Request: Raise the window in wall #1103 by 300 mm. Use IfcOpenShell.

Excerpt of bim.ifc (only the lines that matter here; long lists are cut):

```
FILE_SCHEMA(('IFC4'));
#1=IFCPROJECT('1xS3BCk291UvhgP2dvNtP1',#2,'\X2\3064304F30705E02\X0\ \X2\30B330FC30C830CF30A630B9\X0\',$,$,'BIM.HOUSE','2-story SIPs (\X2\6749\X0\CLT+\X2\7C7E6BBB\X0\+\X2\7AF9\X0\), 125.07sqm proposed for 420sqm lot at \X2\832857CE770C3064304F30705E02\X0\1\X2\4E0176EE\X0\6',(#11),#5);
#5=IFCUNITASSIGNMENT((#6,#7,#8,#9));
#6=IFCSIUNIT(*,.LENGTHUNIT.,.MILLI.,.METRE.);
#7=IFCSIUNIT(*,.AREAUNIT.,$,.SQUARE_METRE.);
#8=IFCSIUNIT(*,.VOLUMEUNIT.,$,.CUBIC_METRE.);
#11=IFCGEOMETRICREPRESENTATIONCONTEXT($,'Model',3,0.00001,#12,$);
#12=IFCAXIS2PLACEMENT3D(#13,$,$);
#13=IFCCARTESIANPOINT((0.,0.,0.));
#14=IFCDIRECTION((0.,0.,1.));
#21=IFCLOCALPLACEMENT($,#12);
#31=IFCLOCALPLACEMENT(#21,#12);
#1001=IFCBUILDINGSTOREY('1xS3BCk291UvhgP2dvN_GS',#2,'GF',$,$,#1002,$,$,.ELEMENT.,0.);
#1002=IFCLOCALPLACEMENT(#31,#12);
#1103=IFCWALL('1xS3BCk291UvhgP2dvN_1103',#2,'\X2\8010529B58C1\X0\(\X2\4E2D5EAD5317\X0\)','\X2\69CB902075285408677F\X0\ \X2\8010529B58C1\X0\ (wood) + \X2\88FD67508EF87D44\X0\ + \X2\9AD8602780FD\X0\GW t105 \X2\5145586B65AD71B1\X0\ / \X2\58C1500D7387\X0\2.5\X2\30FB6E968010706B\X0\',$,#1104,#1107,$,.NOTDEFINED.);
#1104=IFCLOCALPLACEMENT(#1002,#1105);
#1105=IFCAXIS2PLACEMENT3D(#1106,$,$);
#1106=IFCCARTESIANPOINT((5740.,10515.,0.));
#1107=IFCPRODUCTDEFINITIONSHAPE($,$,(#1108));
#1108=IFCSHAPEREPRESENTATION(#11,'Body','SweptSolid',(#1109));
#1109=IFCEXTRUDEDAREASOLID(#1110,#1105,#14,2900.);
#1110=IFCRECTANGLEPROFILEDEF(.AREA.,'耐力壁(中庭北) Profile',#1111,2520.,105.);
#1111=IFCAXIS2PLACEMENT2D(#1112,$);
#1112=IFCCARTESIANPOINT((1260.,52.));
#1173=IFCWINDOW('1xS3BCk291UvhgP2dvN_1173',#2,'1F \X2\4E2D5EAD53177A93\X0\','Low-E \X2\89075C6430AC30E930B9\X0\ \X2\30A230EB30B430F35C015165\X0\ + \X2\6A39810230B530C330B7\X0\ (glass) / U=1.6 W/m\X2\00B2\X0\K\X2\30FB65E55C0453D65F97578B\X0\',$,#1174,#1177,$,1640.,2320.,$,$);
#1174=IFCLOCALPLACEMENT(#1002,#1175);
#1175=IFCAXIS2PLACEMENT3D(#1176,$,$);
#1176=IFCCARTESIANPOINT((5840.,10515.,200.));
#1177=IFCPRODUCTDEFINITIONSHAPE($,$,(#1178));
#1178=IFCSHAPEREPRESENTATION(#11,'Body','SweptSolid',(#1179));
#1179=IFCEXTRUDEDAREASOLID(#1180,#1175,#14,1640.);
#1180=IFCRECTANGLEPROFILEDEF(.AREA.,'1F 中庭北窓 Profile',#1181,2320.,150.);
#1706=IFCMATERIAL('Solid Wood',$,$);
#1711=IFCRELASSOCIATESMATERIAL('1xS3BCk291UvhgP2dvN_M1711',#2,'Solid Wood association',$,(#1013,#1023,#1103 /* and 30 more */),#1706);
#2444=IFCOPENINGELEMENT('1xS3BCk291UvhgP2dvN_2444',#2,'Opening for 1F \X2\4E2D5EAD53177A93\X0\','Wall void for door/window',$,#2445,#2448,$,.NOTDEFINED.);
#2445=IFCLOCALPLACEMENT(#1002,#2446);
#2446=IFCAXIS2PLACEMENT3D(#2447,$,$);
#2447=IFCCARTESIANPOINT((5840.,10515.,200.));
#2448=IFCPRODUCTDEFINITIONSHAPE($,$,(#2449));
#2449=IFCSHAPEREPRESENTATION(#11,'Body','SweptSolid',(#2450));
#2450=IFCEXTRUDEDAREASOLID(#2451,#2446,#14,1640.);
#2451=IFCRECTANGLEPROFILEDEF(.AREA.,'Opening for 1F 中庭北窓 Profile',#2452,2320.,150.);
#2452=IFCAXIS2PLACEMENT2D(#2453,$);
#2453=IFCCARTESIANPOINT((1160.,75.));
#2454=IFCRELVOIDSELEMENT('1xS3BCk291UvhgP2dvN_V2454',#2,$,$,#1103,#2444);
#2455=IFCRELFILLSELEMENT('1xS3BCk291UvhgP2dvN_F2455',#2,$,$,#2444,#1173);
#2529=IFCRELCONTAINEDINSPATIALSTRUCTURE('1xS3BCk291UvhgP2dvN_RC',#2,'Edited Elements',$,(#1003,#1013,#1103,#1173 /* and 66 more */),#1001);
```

```python
import numpy as np
import ifcopenshell
import ifcopenshell.api.geometry
import ifcopenshell.util.placement
import ifcopenshell.util.unit

model = ifcopenshell.open("bim.ifc")
unit_scale = ifcopenshell.util.unit.calculate_unit_scale(model)

window = model.by_guid("1xS3BCk291UvhgP2dvN_1173")
opening = window.FillsVoids[0].RelatingOpeningElement
dz = 300.0

shift = np.array([0.0, 0.0, dz])
# The window is not placed relative to its opening, so move both.
for product in (opening, window):
    matrix = ifcopenshell.util.placement.get_local_placement(product.ObjectPlacement)
    matrix[:3, 3] += shift
    ifcopenshell.api.geometry.edit_object_placement(model, product=product, matrix=matrix, is_si=False)

print(f"moved by {dz * unit_scale:+.3f} m")

model.write("bim_updated.ifc")
```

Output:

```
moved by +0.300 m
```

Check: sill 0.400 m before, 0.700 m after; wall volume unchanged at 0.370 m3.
